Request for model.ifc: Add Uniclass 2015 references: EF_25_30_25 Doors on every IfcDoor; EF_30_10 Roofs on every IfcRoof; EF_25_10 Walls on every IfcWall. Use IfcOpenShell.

First a look at what the model holds.

```python
import ifcopenshell

model = ifcopenshell.open("model.ifc")
print(model.schema)
print("classifications:", [c.Name for c in model.by_type("IfcClassification")])
for ifc_class in ("IfcDoor", "IfcRoof", "IfcStair", "IfcWall", "IfcWindow"):
    print(ifc_class, len(model.by_type(ifc_class)))
```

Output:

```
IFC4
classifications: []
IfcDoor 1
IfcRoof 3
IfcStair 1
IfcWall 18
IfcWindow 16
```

```python
import ifcopenshell
import ifcopenshell.api.classification

model = ifcopenshell.open("model.ifc")

system = ifcopenshell.api.classification.add_classification(model, classification="Uniclass 2015")

codes = {
    "IfcDoor": ("EF_25_30_25", "Doors"),
    "IfcRoof": ("EF_30_10", "Roofs"),
    "IfcWall": ("EF_25_10", "Walls"),
}
for ifc_class, (code, name) in codes.items():
    products = model.by_type(ifc_class)
    ifcopenshell.api.classification.add_reference(
        model, products=products, classification=system, identification=code, name=name
    )
    print(code, len(products))

model.write("model_updated.ifc")
```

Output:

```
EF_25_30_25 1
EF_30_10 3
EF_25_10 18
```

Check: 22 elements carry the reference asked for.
